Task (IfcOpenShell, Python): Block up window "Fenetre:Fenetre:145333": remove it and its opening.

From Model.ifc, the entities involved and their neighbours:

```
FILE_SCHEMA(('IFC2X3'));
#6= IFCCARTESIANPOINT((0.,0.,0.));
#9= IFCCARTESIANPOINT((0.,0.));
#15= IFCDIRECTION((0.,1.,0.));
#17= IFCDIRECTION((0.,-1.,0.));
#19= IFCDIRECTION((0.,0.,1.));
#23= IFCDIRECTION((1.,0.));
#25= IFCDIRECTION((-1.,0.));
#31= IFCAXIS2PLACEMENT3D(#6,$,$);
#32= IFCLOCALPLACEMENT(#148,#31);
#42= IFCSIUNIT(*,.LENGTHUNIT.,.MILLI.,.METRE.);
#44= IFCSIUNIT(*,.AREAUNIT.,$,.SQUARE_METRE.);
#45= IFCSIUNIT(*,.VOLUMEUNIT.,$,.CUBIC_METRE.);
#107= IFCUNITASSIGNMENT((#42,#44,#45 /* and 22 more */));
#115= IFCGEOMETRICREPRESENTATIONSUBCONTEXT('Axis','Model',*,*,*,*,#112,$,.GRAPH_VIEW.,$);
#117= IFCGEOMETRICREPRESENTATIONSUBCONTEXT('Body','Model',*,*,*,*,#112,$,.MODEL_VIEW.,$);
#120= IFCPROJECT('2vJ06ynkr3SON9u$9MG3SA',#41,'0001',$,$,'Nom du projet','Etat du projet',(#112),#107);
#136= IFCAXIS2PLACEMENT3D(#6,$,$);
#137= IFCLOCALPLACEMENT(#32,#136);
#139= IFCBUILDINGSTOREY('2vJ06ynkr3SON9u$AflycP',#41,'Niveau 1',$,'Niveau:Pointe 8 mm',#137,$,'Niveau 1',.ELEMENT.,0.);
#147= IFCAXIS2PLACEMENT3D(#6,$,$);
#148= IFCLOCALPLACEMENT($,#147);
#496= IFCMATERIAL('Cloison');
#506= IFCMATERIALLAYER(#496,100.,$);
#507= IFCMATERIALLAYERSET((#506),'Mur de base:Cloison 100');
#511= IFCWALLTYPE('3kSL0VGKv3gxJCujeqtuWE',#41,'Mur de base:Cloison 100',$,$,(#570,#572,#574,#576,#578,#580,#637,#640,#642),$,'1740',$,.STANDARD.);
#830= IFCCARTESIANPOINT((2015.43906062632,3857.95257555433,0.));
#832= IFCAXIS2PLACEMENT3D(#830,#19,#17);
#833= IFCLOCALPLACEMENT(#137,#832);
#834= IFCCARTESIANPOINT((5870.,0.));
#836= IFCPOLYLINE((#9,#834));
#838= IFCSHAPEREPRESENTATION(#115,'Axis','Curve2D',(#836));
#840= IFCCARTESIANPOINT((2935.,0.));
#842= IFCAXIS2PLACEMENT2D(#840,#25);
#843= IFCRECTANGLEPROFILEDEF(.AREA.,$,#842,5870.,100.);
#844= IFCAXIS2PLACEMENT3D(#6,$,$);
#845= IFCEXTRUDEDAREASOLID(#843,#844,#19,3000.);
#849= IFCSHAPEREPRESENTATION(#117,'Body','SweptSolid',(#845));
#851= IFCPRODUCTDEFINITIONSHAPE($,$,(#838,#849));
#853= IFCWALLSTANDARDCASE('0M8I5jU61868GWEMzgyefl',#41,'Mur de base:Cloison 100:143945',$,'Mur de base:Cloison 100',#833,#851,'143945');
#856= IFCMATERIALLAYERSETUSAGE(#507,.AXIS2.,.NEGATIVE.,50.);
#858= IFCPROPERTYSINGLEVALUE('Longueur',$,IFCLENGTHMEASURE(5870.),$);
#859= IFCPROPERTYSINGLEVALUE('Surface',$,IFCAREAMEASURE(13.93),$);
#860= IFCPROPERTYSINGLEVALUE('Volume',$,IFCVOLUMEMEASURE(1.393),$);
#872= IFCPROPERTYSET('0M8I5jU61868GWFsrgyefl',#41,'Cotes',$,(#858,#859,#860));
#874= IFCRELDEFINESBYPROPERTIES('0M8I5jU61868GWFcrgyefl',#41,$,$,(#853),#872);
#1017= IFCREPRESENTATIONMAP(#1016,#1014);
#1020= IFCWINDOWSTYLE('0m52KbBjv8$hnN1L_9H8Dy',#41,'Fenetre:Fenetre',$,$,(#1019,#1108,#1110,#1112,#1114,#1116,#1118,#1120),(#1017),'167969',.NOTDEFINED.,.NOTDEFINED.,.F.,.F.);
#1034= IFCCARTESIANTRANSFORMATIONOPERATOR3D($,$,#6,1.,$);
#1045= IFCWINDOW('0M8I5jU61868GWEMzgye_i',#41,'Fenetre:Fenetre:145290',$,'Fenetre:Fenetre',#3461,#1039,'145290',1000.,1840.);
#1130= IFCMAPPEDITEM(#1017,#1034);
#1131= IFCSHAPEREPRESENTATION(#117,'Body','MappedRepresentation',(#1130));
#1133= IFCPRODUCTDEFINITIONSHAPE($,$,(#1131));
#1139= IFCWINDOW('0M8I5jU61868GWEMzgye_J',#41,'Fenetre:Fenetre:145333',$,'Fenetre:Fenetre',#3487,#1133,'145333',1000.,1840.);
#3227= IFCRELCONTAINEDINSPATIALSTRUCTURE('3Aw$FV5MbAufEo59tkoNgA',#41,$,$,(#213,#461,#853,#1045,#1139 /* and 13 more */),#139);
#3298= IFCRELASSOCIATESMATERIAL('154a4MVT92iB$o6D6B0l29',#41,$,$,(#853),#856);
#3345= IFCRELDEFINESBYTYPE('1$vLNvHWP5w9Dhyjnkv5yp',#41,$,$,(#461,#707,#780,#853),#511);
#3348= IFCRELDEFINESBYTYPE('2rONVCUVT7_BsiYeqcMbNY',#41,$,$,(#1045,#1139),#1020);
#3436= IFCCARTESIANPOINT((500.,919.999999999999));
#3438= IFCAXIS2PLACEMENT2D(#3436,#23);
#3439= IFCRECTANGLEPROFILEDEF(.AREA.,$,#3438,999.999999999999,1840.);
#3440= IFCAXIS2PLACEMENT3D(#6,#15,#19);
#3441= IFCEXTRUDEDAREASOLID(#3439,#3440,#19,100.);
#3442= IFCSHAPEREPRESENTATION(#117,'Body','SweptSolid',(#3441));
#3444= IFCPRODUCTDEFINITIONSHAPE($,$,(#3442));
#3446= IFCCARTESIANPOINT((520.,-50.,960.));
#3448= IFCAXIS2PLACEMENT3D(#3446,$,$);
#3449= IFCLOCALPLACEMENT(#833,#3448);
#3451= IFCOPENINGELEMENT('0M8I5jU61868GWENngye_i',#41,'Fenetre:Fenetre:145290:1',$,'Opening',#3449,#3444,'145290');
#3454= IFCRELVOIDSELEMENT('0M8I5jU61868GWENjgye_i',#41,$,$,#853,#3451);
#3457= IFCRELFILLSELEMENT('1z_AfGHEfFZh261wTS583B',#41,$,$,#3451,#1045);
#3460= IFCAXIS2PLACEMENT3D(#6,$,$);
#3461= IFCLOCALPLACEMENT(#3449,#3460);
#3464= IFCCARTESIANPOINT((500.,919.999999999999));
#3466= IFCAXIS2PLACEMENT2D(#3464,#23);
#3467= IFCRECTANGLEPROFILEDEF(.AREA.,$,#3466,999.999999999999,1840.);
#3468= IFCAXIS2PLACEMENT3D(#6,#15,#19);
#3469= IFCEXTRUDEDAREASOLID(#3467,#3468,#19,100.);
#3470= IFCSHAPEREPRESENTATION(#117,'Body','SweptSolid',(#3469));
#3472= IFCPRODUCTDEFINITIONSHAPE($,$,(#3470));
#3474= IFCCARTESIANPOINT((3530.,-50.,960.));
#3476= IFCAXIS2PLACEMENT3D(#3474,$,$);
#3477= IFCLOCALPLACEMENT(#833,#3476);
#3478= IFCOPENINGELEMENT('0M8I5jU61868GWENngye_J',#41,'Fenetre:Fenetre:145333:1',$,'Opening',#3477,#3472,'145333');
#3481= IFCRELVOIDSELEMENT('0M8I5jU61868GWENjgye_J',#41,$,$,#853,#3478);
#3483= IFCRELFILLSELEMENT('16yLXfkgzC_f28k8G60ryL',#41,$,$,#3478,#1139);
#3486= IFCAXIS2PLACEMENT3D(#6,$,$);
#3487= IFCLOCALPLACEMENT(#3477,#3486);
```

```python
import ifcopenshell
import ifcopenshell.api.feature
import ifcopenshell.api.pset
import ifcopenshell.api.root
import ifcopenshell.geom
import ifcopenshell.util.element
import ifcopenshell.util.shape
import ifcopenshell.util.unit

model = ifcopenshell.open("Model.ifc")
area_scale = ifcopenshell.util.unit.calculate_unit_scale(model, "AREAUNIT")
volume_scale = ifcopenshell.util.unit.calculate_unit_scale(model, "VOLUMEUNIT")
settings = ifcopenshell.geom.settings()


def volume(element):
    """Net volume in cubic metres, openings subtracted."""
    shape = ifcopenshell.geom.create_shape(settings, element)
    return ifcopenshell.util.shape.get_volume(shape.geometry)


window = model.by_guid("0M8I5jU61868GWEMzgye_J")
opening = window.FillsVoids[0].RelatingOpeningElement
wall = opening.VoidsElements[0].RelatingBuildingElement
before = volume(wall)

ifcopenshell.api.root.remove_product(model, product=window)
ifcopenshell.api.feature.remove_feature(model, feature=opening)

after = volume(wall)
thickness = 0.1  # wall thickness in metres

# Update the wall's stored quantities.
pset = model.by_id(ifcopenshell.util.element.get_pset(wall, "Cotes", should_inherit=False)["id"])
ifcopenshell.api.pset.edit_pset(model, pset=pset, properties={
    "Surface": model.create_entity("IfcAreaMeasure", after / thickness / area_scale),
    "Volume": model.create_entity("IfcVolumeMeasure", after / volume_scale),
})

print(f"wall volume {before:.3f} -> {after:.3f} m3")

model.write("Model_updated.ifc")
```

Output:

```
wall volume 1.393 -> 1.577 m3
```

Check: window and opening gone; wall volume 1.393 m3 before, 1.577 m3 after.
